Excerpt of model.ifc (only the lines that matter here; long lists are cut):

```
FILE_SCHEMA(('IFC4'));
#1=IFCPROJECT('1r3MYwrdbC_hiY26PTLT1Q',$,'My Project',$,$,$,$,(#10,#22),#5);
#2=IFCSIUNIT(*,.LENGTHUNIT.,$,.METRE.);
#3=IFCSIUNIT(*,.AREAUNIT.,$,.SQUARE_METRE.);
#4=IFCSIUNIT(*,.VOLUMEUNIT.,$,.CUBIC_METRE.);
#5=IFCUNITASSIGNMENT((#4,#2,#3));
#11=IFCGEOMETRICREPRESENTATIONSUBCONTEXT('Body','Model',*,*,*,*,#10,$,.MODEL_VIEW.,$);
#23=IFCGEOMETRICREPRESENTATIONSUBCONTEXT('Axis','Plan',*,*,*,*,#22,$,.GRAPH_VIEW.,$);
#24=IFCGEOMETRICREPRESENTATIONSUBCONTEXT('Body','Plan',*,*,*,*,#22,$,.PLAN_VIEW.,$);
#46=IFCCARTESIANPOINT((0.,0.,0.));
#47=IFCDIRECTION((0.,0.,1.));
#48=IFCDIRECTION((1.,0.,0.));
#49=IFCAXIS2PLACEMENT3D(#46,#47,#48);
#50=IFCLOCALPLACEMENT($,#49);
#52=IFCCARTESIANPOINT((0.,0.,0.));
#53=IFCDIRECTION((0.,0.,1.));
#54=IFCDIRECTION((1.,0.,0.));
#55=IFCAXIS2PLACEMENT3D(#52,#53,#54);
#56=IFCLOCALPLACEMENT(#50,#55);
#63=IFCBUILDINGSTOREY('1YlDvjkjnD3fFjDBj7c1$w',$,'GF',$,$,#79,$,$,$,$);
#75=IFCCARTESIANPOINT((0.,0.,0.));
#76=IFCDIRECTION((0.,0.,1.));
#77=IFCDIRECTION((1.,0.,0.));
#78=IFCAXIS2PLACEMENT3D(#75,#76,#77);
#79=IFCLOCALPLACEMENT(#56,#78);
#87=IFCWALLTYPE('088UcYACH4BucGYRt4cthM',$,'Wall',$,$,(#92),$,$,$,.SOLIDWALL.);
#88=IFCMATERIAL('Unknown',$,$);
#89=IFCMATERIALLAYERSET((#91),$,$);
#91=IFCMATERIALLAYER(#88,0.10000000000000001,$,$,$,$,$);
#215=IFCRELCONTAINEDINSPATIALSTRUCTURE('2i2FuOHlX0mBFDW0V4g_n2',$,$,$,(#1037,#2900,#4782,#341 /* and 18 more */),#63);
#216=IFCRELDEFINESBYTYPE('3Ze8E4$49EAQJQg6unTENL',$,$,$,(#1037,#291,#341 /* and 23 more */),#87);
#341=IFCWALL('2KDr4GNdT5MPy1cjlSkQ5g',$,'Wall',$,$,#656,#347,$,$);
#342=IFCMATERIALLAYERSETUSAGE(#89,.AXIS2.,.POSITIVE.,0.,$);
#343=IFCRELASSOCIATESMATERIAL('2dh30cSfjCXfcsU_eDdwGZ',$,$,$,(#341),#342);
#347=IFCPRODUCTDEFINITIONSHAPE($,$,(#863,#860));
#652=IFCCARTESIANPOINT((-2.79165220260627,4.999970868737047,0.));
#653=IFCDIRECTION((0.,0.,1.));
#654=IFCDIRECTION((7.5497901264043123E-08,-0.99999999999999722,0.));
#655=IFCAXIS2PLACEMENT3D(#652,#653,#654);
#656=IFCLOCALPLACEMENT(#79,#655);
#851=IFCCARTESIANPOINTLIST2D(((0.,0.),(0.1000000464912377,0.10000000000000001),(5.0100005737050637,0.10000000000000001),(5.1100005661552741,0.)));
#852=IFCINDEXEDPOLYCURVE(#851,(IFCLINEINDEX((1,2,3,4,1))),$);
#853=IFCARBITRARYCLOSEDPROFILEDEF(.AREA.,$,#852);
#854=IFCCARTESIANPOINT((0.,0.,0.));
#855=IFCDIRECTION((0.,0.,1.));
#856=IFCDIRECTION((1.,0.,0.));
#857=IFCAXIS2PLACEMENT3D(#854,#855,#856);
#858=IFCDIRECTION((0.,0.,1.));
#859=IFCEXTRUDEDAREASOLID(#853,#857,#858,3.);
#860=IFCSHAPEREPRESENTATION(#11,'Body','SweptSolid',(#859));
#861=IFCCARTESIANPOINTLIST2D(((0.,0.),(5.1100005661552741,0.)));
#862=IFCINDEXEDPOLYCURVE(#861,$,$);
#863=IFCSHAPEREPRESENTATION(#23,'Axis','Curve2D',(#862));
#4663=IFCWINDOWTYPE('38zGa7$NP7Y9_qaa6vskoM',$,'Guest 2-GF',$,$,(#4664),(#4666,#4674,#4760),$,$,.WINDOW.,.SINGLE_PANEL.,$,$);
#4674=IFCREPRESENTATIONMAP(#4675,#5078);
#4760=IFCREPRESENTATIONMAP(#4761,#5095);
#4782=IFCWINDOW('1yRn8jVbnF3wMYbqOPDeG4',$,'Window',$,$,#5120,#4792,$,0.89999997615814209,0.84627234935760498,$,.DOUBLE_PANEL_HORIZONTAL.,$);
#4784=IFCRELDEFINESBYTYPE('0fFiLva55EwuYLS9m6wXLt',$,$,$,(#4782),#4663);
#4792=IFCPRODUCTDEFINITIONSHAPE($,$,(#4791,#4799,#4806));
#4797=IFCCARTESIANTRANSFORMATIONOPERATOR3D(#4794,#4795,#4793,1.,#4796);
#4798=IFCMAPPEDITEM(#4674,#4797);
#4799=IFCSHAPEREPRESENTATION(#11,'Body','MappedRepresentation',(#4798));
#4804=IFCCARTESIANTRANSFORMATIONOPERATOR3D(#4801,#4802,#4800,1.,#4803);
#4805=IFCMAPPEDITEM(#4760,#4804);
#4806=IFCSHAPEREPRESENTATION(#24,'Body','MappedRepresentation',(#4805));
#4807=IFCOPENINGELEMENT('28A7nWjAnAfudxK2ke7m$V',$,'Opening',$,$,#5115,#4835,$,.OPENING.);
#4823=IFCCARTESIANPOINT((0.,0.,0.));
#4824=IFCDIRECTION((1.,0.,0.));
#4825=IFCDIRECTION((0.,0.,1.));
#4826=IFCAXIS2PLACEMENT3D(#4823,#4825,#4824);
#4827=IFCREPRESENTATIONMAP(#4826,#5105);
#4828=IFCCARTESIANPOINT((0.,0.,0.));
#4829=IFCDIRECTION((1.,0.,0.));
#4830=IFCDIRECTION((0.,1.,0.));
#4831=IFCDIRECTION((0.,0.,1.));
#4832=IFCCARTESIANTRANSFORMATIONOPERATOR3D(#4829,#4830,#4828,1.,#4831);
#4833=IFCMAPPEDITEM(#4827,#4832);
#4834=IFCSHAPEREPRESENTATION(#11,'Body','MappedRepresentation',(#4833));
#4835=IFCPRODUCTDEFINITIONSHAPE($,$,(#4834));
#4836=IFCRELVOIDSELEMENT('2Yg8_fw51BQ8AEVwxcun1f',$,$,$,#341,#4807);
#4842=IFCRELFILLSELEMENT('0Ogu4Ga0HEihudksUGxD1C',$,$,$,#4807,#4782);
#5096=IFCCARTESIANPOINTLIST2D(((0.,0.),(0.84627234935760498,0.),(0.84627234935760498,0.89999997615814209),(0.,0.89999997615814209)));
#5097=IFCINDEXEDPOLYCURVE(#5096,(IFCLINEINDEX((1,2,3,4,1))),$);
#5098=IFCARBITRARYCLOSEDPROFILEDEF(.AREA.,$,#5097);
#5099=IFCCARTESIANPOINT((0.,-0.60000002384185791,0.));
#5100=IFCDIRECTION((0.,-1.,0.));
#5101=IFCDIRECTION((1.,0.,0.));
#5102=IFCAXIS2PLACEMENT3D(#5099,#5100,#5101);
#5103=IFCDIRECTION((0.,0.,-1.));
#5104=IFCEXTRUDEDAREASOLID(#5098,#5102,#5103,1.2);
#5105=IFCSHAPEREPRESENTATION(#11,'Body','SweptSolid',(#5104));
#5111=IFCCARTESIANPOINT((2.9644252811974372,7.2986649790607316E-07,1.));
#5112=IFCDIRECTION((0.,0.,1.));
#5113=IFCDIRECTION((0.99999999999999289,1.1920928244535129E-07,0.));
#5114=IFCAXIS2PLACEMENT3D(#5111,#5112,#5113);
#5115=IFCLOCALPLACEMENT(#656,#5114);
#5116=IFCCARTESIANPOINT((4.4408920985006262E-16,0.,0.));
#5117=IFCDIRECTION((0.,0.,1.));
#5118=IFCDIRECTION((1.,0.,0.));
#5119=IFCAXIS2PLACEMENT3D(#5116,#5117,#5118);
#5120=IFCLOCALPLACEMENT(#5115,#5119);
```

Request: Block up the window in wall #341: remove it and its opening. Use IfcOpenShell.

```python
import ifcopenshell
import ifcopenshell.api.feature
import ifcopenshell.api.root
import ifcopenshell.geom
import ifcopenshell.util.shape

model = ifcopenshell.open("model.ifc")
settings = ifcopenshell.geom.settings()


def volume(element):
    """Net volume in cubic metres, openings subtracted."""
    shape = ifcopenshell.geom.create_shape(settings, element)
    return ifcopenshell.util.shape.get_volume(shape.geometry)


window = model.by_guid("1yRn8jVbnF3wMYbqOPDeG4")
opening = window.FillsVoids[0].RelatingOpeningElement
wall = opening.VoidsElements[0].RelatingBuildingElement
before = volume(wall)

ifcopenshell.api.root.remove_product(model, product=window)
ifcopenshell.api.feature.remove_feature(model, feature=opening)

after = volume(wall)

print(f"wall volume {before:.3f} -> {after:.3f} m3")

model.write("model_updated.ifc")
```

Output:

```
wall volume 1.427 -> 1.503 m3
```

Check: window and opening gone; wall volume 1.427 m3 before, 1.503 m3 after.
